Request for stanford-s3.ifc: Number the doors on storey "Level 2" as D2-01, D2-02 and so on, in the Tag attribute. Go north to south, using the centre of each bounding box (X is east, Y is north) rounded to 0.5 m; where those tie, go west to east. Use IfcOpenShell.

First a look at what the model holds.

```python
import ifcopenshell
import ifcopenshell.util.element
import ifcopenshell.util.placement

model = ifcopenshell.open("stanford-s3.ifc")
print(model.schema)
storey = next(s for s in model.by_type("IfcBuildingStorey") if s.Name == "Level 2")
doors = [e for e in ifcopenshell.util.element.get_decomposition(storey) if e.is_a("IfcDoor")]
for e in sorted(doors, key=lambda e: e.id()):
    origin = ifcopenshell.util.placement.get_local_placement(e.ObjectPlacement)[:3, 3]
    print(e.id(), e.Tag, e.Name, origin.round(2) + 0.0, sep=" | ")
```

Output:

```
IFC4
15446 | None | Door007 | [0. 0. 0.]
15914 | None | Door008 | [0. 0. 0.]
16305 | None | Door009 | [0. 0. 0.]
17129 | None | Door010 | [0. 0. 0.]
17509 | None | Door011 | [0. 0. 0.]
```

```python
import ifcopenshell
import ifcopenshell.geom
import ifcopenshell.util.element
import ifcopenshell.util.shape

model = ifcopenshell.open("stanford-s3.ifc")
settings = ifcopenshell.geom.settings()
settings.set("use-world-coords", True)


def centre(element):
    shape = ifcopenshell.geom.create_shape(settings, element)
    return ifcopenshell.util.shape.get_bbox_centroid(shape.geometry)


storey = next(s for s in model.by_type("IfcBuildingStorey") if s.Name == "Level 2")
doors = [e for e in ifcopenshell.util.element.get_decomposition(storey) if e.is_a("IfcDoor")]

# Insertion points can sit at a corner or the storey origin, so sort by the geometry (in metres).
centres = {e: centre(e) for e in doors}
doors.sort(key=lambda e: (-round(centres[e][1] / 0.5), centres[e][0]))

for i, e in enumerate(doors, start=1):
    number = f"D2-{i:02d}"
    e.Tag = number
    print(e.id(), number)

model.write("stanford-s3_updated.ifc")
```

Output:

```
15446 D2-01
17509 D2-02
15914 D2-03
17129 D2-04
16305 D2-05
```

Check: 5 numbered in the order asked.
